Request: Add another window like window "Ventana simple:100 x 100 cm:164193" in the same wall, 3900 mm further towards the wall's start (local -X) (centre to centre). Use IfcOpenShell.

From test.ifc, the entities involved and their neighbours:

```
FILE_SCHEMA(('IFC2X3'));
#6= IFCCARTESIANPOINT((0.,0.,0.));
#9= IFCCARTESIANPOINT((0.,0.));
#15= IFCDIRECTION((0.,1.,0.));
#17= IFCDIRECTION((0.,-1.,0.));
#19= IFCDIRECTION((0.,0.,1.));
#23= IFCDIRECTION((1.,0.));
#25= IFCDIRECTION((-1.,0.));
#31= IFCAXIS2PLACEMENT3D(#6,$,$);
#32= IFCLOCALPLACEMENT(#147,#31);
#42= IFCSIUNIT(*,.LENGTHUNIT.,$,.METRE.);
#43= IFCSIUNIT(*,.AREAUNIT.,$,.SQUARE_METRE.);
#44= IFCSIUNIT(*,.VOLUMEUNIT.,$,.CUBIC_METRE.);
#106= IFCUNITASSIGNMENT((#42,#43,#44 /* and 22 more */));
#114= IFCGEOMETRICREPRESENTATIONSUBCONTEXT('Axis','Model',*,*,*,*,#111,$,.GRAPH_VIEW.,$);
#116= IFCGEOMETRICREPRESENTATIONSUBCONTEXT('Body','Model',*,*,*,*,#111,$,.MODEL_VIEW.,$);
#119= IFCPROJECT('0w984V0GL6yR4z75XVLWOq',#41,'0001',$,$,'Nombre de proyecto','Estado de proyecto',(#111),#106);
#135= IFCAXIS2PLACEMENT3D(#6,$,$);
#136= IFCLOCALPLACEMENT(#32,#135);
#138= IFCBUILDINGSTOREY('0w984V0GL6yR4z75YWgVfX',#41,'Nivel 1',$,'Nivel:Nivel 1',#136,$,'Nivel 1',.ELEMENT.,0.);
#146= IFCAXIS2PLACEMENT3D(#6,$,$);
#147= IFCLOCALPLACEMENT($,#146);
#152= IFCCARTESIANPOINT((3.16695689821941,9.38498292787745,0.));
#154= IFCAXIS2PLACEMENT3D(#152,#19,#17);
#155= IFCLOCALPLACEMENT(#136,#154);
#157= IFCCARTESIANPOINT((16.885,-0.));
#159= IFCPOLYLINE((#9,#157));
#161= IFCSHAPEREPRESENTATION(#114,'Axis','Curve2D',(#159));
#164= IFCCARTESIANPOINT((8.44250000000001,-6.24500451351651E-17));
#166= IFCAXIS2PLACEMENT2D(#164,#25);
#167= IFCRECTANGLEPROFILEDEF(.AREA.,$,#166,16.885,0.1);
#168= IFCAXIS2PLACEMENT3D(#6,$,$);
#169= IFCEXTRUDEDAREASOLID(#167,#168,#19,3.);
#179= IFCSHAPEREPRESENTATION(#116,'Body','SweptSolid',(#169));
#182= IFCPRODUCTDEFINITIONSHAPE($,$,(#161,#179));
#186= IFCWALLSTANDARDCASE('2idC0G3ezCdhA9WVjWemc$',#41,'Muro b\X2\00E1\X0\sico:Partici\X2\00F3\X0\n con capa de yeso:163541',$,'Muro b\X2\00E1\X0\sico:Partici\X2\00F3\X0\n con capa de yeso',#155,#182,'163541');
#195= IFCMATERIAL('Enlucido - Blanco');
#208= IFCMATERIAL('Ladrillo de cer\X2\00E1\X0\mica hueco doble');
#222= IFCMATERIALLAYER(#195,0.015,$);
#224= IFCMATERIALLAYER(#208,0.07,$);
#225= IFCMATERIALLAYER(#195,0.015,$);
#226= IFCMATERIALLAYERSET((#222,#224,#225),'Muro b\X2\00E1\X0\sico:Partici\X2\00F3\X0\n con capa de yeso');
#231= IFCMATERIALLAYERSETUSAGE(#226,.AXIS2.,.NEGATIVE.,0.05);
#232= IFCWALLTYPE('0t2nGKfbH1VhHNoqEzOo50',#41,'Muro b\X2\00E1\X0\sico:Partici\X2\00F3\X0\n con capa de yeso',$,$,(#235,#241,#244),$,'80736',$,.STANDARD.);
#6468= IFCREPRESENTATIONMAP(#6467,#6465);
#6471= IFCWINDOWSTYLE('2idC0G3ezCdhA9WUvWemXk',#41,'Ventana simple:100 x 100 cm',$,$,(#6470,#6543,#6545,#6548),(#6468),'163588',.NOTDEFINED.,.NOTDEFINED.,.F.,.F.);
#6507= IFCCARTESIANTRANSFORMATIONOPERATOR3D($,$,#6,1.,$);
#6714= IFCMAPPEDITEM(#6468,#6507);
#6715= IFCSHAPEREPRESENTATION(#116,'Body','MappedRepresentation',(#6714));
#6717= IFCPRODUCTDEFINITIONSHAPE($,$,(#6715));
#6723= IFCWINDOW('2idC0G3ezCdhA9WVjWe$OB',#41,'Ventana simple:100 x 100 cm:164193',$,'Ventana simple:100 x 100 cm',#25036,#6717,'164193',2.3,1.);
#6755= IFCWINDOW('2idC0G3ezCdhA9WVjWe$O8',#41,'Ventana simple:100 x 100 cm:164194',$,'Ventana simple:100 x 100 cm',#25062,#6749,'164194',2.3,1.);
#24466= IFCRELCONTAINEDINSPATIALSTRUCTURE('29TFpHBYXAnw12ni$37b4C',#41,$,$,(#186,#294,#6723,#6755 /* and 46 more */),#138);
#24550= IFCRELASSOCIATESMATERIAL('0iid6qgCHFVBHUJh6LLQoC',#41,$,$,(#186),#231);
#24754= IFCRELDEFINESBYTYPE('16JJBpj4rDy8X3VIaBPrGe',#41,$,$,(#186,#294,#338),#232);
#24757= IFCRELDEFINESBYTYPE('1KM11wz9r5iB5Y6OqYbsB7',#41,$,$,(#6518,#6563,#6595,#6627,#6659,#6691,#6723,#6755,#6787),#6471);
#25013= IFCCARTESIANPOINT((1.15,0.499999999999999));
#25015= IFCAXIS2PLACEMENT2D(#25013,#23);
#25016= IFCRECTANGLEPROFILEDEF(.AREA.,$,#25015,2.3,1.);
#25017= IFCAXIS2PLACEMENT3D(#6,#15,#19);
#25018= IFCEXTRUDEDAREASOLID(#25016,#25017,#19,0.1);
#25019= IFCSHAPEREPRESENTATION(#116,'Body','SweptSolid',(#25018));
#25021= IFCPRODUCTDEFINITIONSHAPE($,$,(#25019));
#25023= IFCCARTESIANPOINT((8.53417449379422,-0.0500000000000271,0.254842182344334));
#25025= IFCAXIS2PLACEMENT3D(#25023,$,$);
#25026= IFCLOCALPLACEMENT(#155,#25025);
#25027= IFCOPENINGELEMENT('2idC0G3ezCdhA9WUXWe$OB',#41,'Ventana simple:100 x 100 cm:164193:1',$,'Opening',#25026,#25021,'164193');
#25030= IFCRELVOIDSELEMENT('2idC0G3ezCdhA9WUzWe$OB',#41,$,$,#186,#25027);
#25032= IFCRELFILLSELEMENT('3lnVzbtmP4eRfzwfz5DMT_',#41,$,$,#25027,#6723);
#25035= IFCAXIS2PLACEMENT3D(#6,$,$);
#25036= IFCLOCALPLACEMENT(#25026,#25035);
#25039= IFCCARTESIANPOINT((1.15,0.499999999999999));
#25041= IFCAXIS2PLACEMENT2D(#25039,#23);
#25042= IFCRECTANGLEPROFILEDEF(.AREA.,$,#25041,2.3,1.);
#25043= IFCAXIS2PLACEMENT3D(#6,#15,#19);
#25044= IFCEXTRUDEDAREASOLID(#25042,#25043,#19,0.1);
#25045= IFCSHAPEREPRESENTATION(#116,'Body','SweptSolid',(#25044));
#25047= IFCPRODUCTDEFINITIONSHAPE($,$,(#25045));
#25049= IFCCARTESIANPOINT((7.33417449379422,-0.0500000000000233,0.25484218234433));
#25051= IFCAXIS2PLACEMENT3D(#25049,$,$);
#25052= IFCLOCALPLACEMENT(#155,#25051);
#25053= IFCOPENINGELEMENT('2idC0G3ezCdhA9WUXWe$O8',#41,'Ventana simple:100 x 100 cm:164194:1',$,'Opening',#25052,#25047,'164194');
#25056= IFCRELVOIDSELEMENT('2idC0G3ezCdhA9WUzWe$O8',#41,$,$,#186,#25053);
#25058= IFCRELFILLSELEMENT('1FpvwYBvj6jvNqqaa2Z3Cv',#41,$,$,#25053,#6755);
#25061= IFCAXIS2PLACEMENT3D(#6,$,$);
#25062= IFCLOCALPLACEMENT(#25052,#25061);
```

```python
import ifcopenshell
import ifcopenshell.api.feature
import ifcopenshell.api.geometry
import ifcopenshell.api.root
import ifcopenshell.geom
import ifcopenshell.util.element
import ifcopenshell.util.placement
import ifcopenshell.util.shape
import ifcopenshell.util.unit

model = ifcopenshell.open("test.ifc")
unit_scale = ifcopenshell.util.unit.calculate_unit_scale(model)
settings = ifcopenshell.geom.settings()


def volume(element):
    """Net volume in cubic metres, openings subtracted."""
    shape = ifcopenshell.geom.create_shape(settings, element)
    return ifcopenshell.util.shape.get_volume(shape.geometry)


def reuse_history(source, copy):
    """copy_class also copies each property set's owner history, people and application; keep the originals."""
    for rel in copy.IsDefinedBy:
        if rel.is_a("IfcRelDefinesByProperties") and (history := rel.RelatingPropertyDefinition.OwnerHistory):
            rel.RelatingPropertyDefinition.OwnerHistory = source.OwnerHistory
            ifcopenshell.util.element.remove_deep2(model, history)


window = model.by_guid("2idC0G3ezCdhA9WVjWe$OB")
opening = window.FillsVoids[0].RelatingOpeningElement
wall = opening.VoidsElements[0].RelatingBuildingElement
before = volume(wall)
shift = ifcopenshell.util.placement.get_local_placement(wall.ObjectPlacement)[:3, 0] * -3.9 / unit_scale

# copy_class copies the void relationship, type, container and properties, but no geometry.
new_opening = ifcopenshell.api.root.copy_class(model, product=opening)
new_opening.Representation = ifcopenshell.util.element.copy_deep(
    model, opening.Representation, exclude=["IfcGeometricRepresentationContext", "IfcRepresentationMap"]
)
new_opening.Name = "Ventana simple:100 x 100 cm"
new_opening.Tag = None
new_window = ifcopenshell.api.root.copy_class(model, product=window)
new_window.Representation = ifcopenshell.util.element.copy_deep(
    model, window.Representation, exclude=["IfcGeometricRepresentationContext", "IfcRepresentationMap"]
)
new_window.Name = "Ventana simple:100 x 100 cm"
new_window.Tag = None
reuse_history(window, new_window)
fills = ifcopenshell.api.feature.add_filling(model, opening=new_opening, element=new_window)
fills.OwnerHistory = new_window.OwnerHistory  # required in IFC2X3

for old, new in ((opening, new_opening), (window, new_window)):
    matrix = ifcopenshell.util.placement.get_local_placement(old.ObjectPlacement)
    matrix[:3, 3] += shift
    ifcopenshell.api.geometry.edit_object_placement(model, product=new, matrix=matrix, is_si=False)

after = volume(wall)

print(f"wall volume {before:.3f} -> {after:.3f} m3")

model.write("test_updated.ifc")
```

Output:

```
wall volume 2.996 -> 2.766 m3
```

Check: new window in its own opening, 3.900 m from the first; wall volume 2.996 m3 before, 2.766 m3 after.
